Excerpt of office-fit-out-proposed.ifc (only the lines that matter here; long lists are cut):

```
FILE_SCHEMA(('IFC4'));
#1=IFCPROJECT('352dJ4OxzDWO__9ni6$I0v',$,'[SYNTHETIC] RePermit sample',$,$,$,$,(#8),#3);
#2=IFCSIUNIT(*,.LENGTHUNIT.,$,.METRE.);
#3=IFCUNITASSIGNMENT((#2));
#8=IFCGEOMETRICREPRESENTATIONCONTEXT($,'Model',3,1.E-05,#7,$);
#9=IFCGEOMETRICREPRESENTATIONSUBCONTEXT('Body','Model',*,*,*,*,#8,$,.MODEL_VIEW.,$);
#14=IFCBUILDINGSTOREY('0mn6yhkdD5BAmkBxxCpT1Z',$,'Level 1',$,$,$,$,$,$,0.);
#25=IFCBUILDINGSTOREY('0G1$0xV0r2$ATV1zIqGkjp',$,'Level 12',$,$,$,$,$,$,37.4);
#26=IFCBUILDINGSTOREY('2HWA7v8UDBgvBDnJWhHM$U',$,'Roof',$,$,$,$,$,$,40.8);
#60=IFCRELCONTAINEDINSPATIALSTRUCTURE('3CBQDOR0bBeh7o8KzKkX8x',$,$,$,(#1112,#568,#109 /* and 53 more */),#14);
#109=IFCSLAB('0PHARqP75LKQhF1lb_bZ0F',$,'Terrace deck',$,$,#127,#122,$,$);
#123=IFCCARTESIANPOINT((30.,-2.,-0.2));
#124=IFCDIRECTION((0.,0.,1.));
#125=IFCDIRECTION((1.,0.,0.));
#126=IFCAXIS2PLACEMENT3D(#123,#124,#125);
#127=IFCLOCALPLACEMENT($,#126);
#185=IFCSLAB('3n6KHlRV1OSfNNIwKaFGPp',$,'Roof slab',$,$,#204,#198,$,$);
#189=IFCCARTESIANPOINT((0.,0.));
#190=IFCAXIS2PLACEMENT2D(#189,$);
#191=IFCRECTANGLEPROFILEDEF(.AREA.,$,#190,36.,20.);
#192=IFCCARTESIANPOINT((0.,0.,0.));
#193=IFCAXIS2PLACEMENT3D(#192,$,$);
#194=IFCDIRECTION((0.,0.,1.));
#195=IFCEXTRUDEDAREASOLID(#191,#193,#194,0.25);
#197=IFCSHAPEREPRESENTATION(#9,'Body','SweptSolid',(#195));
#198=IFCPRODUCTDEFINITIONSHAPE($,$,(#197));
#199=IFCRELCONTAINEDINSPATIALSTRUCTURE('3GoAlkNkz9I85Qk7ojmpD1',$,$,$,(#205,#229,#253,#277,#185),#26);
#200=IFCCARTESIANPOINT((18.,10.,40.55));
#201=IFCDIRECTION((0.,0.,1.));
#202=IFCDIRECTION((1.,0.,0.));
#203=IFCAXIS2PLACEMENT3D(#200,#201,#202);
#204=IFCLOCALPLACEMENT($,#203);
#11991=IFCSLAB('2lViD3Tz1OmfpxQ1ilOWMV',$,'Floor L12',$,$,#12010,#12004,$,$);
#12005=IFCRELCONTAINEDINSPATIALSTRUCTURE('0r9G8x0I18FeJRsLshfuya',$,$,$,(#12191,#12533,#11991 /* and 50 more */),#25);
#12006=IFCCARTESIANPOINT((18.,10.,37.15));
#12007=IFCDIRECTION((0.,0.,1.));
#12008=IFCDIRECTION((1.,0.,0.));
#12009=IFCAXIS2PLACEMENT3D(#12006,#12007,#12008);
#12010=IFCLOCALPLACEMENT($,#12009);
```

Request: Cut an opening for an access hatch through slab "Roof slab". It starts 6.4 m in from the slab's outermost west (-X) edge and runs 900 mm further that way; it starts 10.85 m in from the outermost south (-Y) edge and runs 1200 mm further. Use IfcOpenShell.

```python
import numpy as np
import ifcopenshell
import ifcopenshell.api.feature
import ifcopenshell.api.geometry
import ifcopenshell.api.root
import ifcopenshell.geom
import ifcopenshell.util.placement
import ifcopenshell.util.representation
import ifcopenshell.util.shape
import ifcopenshell.util.unit

model = ifcopenshell.open("office-fit-out-proposed.ifc")
unit_scale = ifcopenshell.util.unit.calculate_unit_scale(model)
settings = ifcopenshell.geom.settings()


def volume(element):
    """Net volume in cubic metres, openings subtracted."""
    shape = ifcopenshell.geom.create_shape(settings, element)
    return ifcopenshell.util.shape.get_volume(shape.geometry)


slab = model.by_guid("3n6KHlRV1OSfNNIwKaFGPp")
before = volume(slab)

# Extent in the slab's own axes, in metres. The edges named are its -X and -Y sides.
slab_shape = ifcopenshell.geom.create_shape(settings, slab)
vertices = ifcopenshell.util.shape.get_vertices(slab_shape.geometry)
x_min, y_min, bottom = vertices.min(axis=0)
top = vertices[:, 2].max()

opening = ifcopenshell.api.root.create_entity(model, ifc_class="IfcOpeningElement", name="Access hatch opening", predefined_type="OPENING")
context = ifcopenshell.util.representation.get_context(model, "Model", "Body", "MODEL_VIEW")
width, depth = 0.9, 1.2
outline = [(0.0, 0.0), (width, 0.0), (width, depth), (0.0, depth), (0.0, 0.0)]
# Overshoot both faces by 50 mm so the cut is clean.
shape = ifcopenshell.api.geometry.add_slab_representation(
    model, context=context, depth=top - bottom + 0.1, polyline=outline
)
ifcopenshell.api.geometry.assign_representation(model, product=opening, representation=shape)

matrix = ifcopenshell.util.placement.get_local_placement(slab.ObjectPlacement)
matrix[:, 3] = matrix @ np.append(np.array([x_min + 6.4, y_min + 10.85, bottom - 0.05]) / unit_scale, 1.0)
ifcopenshell.api.geometry.edit_object_placement(model, product=opening, matrix=matrix, is_si=False)
ifcopenshell.api.feature.add_feature(model, feature=opening, element=slab)

after = volume(slab)

print(f"slab volume {before:.3f} -> {after:.3f} m3")

model.write("office-fit-out-proposed_updated.ifc")
```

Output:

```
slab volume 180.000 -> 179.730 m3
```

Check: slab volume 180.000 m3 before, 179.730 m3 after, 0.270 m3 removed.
